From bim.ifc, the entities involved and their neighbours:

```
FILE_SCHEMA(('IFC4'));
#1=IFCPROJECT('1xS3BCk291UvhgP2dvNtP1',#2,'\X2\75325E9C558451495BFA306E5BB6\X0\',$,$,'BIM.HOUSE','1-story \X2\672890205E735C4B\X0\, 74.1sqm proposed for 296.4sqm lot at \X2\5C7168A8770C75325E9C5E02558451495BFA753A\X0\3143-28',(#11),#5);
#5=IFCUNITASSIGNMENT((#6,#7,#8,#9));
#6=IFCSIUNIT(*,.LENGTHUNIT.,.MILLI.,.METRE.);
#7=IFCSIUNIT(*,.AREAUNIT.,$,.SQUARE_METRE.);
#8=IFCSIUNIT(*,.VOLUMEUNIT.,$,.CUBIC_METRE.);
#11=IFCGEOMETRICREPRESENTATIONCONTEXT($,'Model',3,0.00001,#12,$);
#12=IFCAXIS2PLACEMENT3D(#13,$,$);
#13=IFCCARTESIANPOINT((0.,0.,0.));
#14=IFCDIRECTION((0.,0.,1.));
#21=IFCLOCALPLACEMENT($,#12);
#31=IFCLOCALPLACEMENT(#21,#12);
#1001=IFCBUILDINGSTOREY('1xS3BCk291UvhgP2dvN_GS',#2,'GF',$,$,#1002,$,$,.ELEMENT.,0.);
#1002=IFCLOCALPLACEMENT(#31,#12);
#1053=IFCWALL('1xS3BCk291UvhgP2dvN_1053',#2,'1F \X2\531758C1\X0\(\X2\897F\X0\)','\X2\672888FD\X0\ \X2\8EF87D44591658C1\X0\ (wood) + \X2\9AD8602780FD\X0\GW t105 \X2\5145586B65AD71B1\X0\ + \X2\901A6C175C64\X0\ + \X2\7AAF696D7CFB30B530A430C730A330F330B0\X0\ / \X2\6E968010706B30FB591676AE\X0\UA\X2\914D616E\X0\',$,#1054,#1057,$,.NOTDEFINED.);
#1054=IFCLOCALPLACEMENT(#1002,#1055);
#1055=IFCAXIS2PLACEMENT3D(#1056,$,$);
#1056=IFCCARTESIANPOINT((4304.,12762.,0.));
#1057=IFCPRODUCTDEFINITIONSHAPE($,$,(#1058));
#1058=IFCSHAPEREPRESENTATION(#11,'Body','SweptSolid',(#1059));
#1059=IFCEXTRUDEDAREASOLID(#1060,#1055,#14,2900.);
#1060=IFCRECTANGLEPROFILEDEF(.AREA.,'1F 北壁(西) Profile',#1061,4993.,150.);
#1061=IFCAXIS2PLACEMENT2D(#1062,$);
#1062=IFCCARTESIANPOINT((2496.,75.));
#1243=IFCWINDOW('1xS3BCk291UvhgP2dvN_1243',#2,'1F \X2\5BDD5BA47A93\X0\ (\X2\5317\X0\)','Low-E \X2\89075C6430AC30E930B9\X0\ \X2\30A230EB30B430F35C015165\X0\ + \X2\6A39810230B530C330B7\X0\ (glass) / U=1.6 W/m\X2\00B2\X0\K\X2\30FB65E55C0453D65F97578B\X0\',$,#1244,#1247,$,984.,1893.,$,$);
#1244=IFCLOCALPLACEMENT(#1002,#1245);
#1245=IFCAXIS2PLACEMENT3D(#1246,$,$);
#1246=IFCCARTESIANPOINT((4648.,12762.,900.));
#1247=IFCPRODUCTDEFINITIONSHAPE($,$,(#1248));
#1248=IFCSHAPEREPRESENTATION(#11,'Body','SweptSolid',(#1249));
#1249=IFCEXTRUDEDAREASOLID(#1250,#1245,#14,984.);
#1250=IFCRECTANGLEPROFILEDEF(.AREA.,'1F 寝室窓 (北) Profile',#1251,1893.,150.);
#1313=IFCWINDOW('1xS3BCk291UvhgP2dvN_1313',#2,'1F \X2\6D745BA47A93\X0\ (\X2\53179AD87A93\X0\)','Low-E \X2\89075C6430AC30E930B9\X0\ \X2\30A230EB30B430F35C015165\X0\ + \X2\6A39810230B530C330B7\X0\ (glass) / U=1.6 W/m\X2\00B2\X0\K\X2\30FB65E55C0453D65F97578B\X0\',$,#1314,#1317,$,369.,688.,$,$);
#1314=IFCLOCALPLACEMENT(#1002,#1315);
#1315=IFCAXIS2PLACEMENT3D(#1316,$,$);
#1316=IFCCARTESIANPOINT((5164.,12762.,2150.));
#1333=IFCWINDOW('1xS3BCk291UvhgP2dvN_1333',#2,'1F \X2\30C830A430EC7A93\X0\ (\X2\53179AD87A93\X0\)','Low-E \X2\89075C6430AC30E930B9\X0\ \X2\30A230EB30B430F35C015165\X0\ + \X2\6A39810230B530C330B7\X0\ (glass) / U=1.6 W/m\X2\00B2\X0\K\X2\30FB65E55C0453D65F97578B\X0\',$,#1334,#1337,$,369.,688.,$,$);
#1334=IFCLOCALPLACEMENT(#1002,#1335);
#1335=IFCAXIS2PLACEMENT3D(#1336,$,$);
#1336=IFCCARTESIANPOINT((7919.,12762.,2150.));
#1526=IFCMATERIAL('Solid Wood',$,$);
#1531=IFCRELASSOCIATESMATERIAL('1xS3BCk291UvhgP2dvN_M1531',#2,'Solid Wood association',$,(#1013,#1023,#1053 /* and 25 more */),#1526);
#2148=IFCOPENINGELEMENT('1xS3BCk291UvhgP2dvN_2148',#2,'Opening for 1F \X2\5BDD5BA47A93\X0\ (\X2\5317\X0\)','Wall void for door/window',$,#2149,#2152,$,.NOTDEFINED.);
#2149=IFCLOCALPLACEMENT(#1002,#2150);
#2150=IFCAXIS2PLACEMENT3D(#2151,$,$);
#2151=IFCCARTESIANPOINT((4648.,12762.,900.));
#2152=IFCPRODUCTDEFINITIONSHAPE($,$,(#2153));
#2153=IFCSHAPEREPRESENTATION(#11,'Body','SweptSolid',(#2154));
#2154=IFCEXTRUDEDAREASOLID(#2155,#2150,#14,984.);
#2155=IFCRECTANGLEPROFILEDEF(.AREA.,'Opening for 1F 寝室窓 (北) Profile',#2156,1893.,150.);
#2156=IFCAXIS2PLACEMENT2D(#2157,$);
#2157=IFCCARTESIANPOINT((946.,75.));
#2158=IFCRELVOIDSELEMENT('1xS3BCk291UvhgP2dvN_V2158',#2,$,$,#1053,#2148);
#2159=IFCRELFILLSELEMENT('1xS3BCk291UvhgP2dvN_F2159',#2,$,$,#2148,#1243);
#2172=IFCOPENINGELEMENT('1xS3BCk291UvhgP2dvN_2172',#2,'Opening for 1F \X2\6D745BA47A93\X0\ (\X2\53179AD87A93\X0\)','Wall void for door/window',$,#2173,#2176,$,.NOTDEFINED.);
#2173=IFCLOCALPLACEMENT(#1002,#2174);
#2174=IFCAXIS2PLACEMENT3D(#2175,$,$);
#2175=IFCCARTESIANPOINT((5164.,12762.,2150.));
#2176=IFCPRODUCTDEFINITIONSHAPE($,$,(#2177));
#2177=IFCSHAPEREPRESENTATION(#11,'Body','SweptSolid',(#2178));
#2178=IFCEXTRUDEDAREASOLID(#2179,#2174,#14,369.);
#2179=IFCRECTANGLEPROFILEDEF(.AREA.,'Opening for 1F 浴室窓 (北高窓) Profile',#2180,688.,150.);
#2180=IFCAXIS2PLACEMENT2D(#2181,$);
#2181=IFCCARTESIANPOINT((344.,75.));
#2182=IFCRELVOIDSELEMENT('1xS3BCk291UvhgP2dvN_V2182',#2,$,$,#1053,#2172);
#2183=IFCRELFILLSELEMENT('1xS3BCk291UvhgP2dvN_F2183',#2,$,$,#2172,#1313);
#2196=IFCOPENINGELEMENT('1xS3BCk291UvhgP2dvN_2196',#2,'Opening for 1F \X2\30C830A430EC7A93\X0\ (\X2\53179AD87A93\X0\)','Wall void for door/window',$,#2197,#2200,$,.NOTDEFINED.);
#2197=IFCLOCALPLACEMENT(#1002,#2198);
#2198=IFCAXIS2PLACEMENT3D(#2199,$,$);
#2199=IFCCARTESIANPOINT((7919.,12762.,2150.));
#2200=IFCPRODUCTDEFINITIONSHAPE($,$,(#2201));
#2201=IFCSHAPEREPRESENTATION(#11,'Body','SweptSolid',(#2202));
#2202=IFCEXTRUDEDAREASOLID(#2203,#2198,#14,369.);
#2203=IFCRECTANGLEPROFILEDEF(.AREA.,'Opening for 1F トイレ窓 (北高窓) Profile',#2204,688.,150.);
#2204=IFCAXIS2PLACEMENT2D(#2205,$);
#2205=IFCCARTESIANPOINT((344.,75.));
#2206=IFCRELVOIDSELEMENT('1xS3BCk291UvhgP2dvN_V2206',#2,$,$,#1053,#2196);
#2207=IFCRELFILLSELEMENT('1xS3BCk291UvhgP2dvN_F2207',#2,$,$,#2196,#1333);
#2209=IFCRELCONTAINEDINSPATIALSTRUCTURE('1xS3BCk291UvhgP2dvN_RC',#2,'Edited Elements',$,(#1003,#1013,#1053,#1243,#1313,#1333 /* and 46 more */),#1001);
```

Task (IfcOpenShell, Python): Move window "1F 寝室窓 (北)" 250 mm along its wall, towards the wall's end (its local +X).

```python
import ifcopenshell
import ifcopenshell.api.geometry
import ifcopenshell.util.placement
import ifcopenshell.util.unit

model = ifcopenshell.open("bim.ifc")
unit_scale = ifcopenshell.util.unit.calculate_unit_scale(model)

window = model.by_guid("1xS3BCk291UvhgP2dvN_1243")
opening = window.FillsVoids[0].RelatingOpeningElement
wall = opening.VoidsElements[0].RelatingBuildingElement

wall_matrix = ifcopenshell.util.placement.get_local_placement(wall.ObjectPlacement)
shift = wall_matrix[:3, 0] * 0.25 / unit_scale
before = ifcopenshell.util.placement.get_local_placement(window.ObjectPlacement)[:3, 3].copy()

# The window is not placed relative to its opening, so move both.
for product in (opening, window):
    matrix = ifcopenshell.util.placement.get_local_placement(product.ObjectPlacement)
    matrix[:3, 3] += shift
    ifcopenshell.api.geometry.edit_object_placement(model, product=product, matrix=matrix, is_si=False)

after = ifcopenshell.util.placement.get_local_placement(window.ObjectPlacement)[:3, 3]
print("window moved by", (after - before).round(3) + 0.0)

model.write("bim_rev.ifc")
```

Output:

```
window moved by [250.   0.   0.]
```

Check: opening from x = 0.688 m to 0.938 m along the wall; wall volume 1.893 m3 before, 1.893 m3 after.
